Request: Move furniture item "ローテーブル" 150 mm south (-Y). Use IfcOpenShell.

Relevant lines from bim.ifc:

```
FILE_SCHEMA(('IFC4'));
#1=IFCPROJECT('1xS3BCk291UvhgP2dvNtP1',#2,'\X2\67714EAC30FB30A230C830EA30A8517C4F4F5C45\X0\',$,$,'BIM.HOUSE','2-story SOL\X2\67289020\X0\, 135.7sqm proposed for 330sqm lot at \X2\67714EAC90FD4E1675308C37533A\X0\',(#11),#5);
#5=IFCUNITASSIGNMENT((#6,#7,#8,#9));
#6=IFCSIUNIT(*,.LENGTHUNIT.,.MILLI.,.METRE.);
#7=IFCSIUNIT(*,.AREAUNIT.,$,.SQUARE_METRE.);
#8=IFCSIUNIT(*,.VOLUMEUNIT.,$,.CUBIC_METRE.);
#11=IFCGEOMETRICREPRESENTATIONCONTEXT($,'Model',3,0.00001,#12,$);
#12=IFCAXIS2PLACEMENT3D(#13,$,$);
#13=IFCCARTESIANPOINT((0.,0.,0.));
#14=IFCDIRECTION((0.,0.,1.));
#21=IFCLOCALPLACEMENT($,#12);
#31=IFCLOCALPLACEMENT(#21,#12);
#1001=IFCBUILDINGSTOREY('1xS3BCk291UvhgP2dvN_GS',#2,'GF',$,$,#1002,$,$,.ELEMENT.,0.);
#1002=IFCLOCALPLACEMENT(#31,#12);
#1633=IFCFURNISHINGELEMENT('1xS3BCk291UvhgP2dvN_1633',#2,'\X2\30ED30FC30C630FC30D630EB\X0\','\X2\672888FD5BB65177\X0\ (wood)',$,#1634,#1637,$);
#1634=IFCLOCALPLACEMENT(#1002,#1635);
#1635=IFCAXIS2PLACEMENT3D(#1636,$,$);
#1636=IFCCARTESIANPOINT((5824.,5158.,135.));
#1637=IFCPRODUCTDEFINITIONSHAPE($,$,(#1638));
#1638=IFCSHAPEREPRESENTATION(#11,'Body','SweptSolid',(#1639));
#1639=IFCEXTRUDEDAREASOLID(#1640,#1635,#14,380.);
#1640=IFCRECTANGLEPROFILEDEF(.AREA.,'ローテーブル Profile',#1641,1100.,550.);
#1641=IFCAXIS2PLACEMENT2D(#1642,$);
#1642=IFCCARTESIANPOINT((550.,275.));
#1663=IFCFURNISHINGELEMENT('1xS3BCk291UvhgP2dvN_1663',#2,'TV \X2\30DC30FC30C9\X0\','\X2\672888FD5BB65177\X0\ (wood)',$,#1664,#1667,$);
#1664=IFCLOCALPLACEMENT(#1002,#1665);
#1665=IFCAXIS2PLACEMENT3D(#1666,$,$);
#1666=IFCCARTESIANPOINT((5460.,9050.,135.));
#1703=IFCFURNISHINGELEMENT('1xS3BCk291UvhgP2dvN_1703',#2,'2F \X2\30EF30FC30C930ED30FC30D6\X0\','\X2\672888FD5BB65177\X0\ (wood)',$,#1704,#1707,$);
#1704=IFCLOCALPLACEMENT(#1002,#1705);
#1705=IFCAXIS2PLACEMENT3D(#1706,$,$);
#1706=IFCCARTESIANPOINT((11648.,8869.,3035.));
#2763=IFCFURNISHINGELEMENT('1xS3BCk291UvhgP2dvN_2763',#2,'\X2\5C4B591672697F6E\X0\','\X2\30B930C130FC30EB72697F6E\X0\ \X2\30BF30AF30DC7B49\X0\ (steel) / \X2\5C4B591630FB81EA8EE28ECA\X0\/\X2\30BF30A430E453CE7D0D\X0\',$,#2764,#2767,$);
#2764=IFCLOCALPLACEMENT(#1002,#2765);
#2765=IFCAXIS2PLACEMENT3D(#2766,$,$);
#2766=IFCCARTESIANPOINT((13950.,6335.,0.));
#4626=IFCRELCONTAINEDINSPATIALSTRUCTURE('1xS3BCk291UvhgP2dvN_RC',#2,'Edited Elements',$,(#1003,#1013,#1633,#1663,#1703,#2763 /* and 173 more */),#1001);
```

```python
import ifcopenshell
import ifcopenshell.api.geometry
import ifcopenshell.util.placement

model = ifcopenshell.open("bim.ifc")

item = model.by_id(1633)
matrix = ifcopenshell.util.placement.get_local_placement(item.ObjectPlacement)
matrix[1, 3] -= 150.0
ifcopenshell.api.geometry.edit_object_placement(model, product=item, matrix=matrix, is_si=False)

print(ifcopenshell.util.placement.get_local_placement(item.ObjectPlacement).round(3) + 0.0)

model.write("bim_rev.ifc")
```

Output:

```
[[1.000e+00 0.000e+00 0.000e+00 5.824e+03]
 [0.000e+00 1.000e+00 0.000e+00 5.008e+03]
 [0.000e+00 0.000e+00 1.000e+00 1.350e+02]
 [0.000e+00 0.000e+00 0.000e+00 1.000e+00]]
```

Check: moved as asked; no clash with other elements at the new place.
